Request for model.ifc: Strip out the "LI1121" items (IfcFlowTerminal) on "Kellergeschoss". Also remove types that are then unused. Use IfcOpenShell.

First a look at what the model holds.

```python
import ifcopenshell
import ifcopenshell.util.element

model = ifcopenshell.open("model.ifc")
print(model.schema)
storey = next(s for s in model.by_type("IfcBuildingStorey") if s.Name == "Kellergeschoss")
terminals = [e for e in ifcopenshell.util.element.get_decomposition(storey) if e.is_a("IfcFlowTerminal")]
seen = {}
for e in terminals:
    element_type = ifcopenshell.util.element.get_type(e)
    name = element_type.Name if element_type not in (None, e) else None
    seen[name] = seen.get(name, 0) + 1
for name, count in sorted(seen.items(), key=str):
    print(count, "x", name)
```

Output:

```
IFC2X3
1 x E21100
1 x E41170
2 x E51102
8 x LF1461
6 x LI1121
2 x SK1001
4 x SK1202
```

```python
import ifcopenshell
import ifcopenshell.api.root
import ifcopenshell.util.element

model = ifcopenshell.open("model.ifc")

storey = next(s for s in model.by_type("IfcBuildingStorey") if s.Name == "Kellergeschoss")
terminals = [e for e in ifcopenshell.util.element.get_decomposition(storey) if e.is_a("IfcFlowTerminal")]
targets = [e for e in terminals if (t := ifcopenshell.util.element.get_type(e)) not in (None, e) and t.Name == "LI1121"]
types = {ifcopenshell.util.element.get_type(e) for e in targets} - {None, *targets}

for e in targets:
    ifcopenshell.api.root.remove_product(model, product=e)
print(len(targets), "removed")

unused = [t for t in types if not ifcopenshell.util.element.get_types(t)]
for t in unused:
    ifcopenshell.api.root.remove_product(model, product=t)
print(len(unused), "unused types removed")

model.write("model-out.ifc")
```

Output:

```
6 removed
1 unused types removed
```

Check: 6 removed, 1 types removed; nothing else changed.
